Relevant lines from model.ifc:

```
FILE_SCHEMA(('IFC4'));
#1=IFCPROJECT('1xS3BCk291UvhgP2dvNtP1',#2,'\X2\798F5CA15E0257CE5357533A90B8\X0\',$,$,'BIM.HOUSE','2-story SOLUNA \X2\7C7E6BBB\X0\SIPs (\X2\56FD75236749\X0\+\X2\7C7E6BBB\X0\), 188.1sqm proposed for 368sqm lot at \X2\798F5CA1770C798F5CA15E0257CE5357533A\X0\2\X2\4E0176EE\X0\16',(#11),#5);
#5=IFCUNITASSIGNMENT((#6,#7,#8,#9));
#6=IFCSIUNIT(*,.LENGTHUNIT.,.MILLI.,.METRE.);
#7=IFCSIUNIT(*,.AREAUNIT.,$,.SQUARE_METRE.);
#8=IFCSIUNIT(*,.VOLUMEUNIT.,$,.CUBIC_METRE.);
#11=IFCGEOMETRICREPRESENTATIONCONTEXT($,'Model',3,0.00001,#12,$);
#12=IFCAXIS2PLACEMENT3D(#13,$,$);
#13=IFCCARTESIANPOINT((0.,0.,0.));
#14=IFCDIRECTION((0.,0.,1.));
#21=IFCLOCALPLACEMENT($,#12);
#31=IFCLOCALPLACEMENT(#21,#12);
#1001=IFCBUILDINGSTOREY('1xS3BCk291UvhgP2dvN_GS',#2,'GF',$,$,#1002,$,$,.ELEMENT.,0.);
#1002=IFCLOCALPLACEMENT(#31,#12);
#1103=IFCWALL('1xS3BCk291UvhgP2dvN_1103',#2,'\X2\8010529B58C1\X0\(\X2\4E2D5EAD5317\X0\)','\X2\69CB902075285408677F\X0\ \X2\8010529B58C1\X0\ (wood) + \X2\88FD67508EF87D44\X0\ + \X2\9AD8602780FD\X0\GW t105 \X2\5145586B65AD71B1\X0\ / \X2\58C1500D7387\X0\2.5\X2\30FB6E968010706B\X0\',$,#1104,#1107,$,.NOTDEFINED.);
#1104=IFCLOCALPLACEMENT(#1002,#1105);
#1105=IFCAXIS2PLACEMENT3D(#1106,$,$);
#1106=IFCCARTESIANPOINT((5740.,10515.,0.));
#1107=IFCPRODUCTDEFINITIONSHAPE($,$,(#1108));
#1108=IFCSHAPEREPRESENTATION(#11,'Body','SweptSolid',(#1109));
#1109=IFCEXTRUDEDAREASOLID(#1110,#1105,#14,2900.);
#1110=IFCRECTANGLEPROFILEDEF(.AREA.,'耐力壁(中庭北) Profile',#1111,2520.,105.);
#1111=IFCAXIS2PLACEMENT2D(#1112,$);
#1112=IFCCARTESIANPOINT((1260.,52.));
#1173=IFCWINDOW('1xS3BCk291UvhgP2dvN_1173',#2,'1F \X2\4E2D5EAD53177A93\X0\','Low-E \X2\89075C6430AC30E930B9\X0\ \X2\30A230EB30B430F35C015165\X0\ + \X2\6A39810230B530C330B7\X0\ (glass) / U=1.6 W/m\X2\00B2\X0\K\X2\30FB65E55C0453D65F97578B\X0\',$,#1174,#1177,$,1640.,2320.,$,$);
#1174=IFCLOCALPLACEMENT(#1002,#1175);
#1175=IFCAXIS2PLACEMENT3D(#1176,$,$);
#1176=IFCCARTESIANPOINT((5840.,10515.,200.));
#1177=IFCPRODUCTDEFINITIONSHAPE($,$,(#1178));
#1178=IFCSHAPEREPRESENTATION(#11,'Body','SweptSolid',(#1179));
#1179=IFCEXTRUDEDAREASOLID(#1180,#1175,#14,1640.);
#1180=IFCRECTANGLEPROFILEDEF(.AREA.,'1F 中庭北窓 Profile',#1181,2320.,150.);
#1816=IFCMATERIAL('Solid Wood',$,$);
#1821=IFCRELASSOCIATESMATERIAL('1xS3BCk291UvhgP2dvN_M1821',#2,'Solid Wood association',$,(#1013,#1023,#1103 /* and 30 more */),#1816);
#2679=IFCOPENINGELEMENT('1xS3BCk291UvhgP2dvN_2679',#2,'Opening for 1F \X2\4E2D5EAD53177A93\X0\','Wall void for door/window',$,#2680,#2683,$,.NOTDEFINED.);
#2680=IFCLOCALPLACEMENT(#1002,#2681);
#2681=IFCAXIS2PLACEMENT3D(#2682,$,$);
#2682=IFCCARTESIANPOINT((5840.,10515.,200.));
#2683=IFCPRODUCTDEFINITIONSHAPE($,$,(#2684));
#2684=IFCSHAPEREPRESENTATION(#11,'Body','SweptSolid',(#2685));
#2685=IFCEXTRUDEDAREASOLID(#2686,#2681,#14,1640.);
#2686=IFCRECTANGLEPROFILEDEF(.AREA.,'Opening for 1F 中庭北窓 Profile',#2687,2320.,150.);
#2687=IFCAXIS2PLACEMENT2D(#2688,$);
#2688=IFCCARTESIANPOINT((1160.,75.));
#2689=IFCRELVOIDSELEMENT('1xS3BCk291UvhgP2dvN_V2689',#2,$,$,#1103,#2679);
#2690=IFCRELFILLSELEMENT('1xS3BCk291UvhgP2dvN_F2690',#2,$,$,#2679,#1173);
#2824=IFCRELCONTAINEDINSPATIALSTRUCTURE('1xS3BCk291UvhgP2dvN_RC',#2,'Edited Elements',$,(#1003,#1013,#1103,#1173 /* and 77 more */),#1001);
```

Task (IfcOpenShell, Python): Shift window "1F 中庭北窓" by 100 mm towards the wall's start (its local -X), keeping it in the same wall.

```python
import ifcopenshell
import ifcopenshell.api.geometry
import ifcopenshell.util.placement
import ifcopenshell.util.unit

model = ifcopenshell.open("model.ifc")
unit_scale = ifcopenshell.util.unit.calculate_unit_scale(model)

window = model.by_id(1173)
opening = window.FillsVoids[0].RelatingOpeningElement
wall = opening.VoidsElements[0].RelatingBuildingElement

wall_matrix = ifcopenshell.util.placement.get_local_placement(wall.ObjectPlacement)
shift = wall_matrix[:3, 0] * -0.1 / unit_scale
before = ifcopenshell.util.placement.get_local_placement(window.ObjectPlacement)[:3, 3].copy()

# The window is not placed relative to its opening, so move both.
for product in (opening, window):
    matrix = ifcopenshell.util.placement.get_local_placement(product.ObjectPlacement)
    matrix[:3, 3] += shift
    ifcopenshell.api.geometry.edit_object_placement(model, product=product, matrix=matrix, is_si=False)

after = ifcopenshell.util.placement.get_local_placement(window.ObjectPlacement)[:3, 3]
print("window moved by", (after - before).round(3) + 0.0)

model.write("model_edited.ifc")
```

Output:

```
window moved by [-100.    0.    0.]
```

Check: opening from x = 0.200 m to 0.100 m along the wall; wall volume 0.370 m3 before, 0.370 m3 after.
